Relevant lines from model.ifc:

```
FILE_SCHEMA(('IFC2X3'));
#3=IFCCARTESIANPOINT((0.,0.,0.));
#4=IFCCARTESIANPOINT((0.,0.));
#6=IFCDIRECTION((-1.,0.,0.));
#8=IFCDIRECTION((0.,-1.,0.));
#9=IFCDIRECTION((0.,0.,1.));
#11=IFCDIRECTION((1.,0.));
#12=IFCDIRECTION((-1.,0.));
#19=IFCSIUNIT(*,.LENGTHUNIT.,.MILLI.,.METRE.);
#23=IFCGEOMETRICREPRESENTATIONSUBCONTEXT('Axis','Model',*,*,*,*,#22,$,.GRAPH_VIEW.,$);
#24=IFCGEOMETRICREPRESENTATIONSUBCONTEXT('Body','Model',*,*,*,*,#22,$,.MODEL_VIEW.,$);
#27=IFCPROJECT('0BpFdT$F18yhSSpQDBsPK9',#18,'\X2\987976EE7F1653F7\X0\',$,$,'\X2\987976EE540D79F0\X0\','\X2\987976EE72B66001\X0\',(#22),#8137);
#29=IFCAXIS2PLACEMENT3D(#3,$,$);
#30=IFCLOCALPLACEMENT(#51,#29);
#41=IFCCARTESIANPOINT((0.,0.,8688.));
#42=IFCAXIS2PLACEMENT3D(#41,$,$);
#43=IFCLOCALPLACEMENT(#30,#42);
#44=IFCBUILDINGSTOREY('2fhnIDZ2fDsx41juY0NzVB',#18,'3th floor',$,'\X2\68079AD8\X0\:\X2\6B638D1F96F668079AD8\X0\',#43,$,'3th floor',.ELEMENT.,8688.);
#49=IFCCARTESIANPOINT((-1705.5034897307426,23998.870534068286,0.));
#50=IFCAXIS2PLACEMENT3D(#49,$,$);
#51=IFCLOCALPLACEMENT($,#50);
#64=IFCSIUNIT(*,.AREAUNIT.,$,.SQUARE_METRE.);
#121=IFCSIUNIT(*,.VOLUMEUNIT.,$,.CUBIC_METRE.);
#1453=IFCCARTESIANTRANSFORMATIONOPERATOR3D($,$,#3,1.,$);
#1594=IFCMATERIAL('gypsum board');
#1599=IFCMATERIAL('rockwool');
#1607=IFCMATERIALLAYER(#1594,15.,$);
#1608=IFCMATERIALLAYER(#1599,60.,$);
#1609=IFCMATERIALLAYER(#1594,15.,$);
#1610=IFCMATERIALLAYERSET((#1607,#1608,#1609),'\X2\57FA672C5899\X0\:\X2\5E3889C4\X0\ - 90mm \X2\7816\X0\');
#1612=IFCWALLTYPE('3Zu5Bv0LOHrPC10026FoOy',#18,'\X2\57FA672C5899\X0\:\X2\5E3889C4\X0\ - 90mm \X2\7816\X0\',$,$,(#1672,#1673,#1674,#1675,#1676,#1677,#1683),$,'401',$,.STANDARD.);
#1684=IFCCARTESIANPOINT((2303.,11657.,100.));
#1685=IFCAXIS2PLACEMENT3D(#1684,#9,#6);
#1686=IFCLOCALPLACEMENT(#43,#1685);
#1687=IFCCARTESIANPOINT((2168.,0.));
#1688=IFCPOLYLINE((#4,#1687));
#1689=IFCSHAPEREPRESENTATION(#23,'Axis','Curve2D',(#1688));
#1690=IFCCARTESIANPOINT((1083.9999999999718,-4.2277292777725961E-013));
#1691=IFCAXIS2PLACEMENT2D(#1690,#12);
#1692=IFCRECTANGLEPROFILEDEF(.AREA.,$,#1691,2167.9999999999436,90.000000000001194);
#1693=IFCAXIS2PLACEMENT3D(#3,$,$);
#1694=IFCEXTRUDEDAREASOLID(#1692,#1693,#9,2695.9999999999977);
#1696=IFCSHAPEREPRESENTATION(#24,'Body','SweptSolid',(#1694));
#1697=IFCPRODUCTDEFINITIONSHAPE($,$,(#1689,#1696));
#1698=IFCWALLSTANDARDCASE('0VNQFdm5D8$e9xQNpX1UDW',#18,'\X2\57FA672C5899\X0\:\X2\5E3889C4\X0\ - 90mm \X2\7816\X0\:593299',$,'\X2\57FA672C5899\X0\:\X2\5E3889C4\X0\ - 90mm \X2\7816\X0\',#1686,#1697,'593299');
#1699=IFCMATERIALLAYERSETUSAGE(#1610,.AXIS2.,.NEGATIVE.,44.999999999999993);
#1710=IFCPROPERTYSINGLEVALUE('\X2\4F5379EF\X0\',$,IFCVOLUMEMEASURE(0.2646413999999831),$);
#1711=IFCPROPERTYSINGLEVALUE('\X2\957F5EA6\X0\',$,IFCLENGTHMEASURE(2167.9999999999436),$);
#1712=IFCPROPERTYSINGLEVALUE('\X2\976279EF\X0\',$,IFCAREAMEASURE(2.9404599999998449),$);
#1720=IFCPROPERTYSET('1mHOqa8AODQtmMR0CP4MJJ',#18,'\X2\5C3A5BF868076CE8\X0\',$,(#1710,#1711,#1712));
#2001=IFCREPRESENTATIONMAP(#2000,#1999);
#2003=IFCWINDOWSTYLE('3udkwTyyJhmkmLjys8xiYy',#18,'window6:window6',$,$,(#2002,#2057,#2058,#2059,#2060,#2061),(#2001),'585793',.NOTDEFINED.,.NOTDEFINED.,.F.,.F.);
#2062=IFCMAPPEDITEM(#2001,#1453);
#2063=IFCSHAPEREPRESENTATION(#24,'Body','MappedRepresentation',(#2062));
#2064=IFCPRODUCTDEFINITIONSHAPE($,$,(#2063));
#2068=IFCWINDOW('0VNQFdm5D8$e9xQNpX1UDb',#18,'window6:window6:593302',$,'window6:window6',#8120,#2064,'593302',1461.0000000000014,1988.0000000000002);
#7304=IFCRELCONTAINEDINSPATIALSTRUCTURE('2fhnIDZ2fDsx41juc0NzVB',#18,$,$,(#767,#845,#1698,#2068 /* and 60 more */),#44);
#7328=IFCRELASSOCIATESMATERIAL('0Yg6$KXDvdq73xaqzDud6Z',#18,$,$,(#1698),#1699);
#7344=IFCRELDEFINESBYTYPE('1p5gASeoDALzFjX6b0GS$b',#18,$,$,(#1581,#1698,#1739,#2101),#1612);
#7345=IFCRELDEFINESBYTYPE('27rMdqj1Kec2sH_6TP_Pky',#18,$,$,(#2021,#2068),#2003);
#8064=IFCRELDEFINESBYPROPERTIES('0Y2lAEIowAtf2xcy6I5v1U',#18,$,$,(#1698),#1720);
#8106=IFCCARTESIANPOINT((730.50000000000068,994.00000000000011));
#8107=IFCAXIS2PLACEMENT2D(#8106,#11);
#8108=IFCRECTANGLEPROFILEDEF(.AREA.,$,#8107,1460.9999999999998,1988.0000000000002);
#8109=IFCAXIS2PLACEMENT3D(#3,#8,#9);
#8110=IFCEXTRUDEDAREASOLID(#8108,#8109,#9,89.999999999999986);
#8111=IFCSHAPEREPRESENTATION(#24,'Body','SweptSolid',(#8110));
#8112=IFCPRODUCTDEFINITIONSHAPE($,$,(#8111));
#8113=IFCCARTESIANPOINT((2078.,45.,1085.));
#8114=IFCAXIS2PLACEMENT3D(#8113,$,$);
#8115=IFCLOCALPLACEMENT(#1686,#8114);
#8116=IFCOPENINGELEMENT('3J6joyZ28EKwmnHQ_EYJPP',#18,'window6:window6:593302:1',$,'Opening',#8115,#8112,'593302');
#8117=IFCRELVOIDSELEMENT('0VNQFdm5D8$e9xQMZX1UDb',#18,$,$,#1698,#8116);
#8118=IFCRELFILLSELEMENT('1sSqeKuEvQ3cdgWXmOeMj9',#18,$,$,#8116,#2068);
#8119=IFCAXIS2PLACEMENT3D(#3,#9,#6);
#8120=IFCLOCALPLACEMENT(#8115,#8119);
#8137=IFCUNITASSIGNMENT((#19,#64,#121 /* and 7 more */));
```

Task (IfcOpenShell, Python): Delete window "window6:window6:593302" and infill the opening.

```python
import ifcopenshell
import ifcopenshell.api.feature
import ifcopenshell.api.pset
import ifcopenshell.api.root
import ifcopenshell.geom
import ifcopenshell.util.element
import ifcopenshell.util.shape
import ifcopenshell.util.unit

model = ifcopenshell.open("model.ifc")
area_scale = ifcopenshell.util.unit.calculate_unit_scale(model, "AREAUNIT")
volume_scale = ifcopenshell.util.unit.calculate_unit_scale(model, "VOLUMEUNIT")
settings = ifcopenshell.geom.settings()


def volume(element):
    """Net volume in cubic metres, openings subtracted."""
    shape = ifcopenshell.geom.create_shape(settings, element)
    return ifcopenshell.util.shape.get_volume(shape.geometry)


window = model.by_guid("0VNQFdm5D8$e9xQNpX1UDb")
opening = window.FillsVoids[0].RelatingOpeningElement
wall = opening.VoidsElements[0].RelatingBuildingElement
before = volume(wall)

ifcopenshell.api.root.remove_product(model, product=window)
ifcopenshell.api.feature.remove_feature(model, feature=opening)

after = volume(wall)
thickness = 0.09  # wall thickness in metres

# Update the wall's stored quantities.
pset = model.by_id(ifcopenshell.util.element.get_pset(wall, "尺寸标注", should_inherit=False)["id"])
ifcopenshell.api.pset.edit_pset(model, pset=pset, properties={
    "体积": model.create_entity("IfcVolumeMeasure", after / volume_scale),
    "面积": model.create_entity("IfcAreaMeasure", after / thickness / area_scale),
})

print(f"wall volume {before:.3f} -> {after:.3f} m3")

model.write("model-out.ifc")
```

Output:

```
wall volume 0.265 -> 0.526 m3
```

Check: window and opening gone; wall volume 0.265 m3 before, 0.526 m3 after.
